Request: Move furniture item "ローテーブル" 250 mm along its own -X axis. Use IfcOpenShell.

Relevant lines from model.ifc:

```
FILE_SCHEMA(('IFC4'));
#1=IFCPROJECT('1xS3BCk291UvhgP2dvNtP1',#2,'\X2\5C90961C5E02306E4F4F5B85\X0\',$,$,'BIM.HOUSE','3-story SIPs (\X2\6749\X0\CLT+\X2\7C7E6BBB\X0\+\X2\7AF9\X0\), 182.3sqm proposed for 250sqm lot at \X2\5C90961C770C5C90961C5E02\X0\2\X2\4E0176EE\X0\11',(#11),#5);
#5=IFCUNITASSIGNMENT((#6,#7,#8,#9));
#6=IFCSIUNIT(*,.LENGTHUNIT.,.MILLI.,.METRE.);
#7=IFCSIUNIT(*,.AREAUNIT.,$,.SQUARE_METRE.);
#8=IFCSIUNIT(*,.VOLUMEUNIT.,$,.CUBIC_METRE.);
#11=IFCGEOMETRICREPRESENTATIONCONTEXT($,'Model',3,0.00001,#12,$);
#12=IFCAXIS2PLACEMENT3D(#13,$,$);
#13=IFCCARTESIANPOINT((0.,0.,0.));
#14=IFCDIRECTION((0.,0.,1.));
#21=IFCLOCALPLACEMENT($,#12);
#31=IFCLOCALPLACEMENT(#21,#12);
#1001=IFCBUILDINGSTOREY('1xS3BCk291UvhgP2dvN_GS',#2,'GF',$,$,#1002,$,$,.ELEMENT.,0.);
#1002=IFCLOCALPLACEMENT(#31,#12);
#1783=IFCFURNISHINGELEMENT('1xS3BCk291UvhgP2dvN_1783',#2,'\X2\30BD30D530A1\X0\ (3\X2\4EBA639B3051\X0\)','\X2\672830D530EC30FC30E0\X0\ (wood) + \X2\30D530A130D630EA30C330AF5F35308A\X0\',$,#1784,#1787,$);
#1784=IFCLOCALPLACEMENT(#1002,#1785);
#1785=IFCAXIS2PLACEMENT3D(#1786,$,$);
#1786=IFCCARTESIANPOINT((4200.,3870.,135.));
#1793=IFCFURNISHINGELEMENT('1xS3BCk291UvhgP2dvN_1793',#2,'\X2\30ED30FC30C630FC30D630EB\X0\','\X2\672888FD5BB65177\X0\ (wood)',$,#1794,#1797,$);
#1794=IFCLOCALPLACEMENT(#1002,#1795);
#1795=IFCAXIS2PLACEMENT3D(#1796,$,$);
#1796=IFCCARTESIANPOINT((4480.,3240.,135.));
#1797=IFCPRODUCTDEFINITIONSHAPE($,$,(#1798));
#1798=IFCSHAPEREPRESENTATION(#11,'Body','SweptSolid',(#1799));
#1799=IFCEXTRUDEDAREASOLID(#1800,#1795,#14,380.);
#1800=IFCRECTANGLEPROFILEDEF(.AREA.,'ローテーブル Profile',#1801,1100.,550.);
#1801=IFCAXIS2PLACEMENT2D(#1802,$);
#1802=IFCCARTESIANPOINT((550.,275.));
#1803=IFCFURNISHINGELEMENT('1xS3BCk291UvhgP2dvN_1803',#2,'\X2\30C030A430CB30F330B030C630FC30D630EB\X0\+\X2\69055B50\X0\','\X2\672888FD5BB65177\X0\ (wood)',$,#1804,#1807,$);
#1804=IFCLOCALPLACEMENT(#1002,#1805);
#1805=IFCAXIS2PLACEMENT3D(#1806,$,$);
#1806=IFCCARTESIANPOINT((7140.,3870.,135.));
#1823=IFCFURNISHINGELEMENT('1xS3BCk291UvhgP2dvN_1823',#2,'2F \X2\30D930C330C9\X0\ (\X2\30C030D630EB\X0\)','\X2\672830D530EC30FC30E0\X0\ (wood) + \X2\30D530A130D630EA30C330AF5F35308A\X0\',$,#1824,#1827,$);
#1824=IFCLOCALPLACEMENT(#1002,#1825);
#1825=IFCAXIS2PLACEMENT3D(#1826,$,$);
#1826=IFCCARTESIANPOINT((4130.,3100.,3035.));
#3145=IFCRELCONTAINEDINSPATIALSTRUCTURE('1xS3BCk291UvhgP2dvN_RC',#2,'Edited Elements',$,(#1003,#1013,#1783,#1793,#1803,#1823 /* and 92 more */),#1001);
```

```python
import ifcopenshell
import ifcopenshell.api.geometry
import ifcopenshell.util.placement
import ifcopenshell.util.unit

model = ifcopenshell.open("model.ifc")
unit_scale = ifcopenshell.util.unit.calculate_unit_scale(model)

item = model.by_guid("1xS3BCk291UvhgP2dvN_1793")
matrix = ifcopenshell.util.placement.get_local_placement(item.ObjectPlacement)
matrix[:3, 3] -= matrix[:3, 0] * 0.25 / unit_scale
ifcopenshell.api.geometry.edit_object_placement(model, product=item, matrix=matrix, is_si=False)

print(ifcopenshell.util.placement.get_local_placement(item.ObjectPlacement).round(3) + 0.0)

model.write("model-out.ifc")
```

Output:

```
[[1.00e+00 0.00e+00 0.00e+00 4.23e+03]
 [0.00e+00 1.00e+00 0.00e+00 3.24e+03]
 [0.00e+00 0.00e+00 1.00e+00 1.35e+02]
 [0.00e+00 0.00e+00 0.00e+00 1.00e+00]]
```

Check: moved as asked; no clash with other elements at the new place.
